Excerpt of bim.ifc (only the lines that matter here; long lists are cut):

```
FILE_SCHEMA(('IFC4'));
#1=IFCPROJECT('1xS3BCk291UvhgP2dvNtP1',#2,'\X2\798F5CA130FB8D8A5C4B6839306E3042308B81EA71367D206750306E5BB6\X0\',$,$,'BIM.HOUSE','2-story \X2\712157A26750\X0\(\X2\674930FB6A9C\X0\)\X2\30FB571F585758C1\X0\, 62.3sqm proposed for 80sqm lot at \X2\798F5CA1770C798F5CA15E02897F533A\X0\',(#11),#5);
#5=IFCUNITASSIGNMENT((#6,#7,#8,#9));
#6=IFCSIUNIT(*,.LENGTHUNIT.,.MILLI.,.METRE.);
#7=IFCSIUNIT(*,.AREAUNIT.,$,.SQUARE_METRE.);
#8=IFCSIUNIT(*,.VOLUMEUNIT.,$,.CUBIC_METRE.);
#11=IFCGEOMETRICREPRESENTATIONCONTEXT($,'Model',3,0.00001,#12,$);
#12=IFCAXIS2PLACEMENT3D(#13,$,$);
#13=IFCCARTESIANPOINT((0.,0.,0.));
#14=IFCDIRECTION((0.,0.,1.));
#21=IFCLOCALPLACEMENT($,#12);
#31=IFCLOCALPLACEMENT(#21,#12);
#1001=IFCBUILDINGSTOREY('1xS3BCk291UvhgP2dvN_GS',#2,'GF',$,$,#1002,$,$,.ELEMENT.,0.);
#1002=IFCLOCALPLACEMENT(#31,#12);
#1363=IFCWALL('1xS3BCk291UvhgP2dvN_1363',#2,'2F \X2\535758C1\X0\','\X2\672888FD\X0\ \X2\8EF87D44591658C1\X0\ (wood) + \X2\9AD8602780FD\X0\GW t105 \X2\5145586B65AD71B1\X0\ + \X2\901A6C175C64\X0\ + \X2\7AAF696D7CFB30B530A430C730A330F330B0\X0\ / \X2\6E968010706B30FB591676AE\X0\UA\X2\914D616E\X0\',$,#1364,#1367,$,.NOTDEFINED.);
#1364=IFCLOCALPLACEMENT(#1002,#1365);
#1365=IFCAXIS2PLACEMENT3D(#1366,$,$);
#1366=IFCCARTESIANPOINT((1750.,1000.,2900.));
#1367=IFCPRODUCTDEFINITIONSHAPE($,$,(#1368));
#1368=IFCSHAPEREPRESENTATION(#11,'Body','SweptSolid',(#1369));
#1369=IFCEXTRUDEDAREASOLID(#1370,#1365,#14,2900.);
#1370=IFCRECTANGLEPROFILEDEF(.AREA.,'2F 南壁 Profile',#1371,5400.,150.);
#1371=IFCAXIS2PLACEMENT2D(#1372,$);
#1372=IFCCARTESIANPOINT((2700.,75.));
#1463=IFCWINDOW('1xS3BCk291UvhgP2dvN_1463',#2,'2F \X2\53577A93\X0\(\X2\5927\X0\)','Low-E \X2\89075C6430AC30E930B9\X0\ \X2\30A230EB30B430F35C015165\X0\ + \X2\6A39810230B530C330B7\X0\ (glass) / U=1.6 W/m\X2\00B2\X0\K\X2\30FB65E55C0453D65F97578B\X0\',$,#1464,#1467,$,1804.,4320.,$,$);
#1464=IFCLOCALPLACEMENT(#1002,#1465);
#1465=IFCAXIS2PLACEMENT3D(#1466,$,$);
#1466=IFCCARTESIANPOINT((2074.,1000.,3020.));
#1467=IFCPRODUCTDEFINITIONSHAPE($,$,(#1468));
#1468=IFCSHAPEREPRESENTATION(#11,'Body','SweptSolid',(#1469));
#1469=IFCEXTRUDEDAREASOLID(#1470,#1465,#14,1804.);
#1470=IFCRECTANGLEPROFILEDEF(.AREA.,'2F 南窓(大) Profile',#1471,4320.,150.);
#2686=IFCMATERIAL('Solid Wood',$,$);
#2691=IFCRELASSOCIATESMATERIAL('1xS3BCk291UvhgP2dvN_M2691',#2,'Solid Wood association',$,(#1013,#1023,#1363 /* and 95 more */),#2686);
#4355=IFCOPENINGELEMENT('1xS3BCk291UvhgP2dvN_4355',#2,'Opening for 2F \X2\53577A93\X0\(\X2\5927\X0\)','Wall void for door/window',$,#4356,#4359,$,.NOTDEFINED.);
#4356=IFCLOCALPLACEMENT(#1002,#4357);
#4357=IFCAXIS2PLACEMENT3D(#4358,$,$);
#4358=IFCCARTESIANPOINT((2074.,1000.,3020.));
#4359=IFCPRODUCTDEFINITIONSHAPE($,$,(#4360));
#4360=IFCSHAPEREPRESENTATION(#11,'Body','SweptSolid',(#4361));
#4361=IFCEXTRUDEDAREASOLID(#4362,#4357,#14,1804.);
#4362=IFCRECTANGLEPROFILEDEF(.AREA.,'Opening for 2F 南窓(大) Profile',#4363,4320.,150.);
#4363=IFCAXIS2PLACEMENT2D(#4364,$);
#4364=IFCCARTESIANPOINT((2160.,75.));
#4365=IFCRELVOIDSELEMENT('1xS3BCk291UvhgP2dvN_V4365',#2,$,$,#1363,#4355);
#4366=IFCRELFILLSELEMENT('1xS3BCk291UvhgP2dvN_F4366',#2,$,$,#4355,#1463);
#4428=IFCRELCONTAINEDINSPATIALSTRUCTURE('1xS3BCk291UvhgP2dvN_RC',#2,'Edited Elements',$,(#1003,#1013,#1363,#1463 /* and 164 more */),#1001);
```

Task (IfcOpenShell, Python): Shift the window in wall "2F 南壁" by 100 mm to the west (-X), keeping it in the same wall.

```python
import ifcopenshell
import ifcopenshell.api.geometry
import ifcopenshell.util.placement

model = ifcopenshell.open("bim.ifc")

window = model.by_guid("1xS3BCk291UvhgP2dvN_1463")
opening = window.FillsVoids[0].RelatingOpeningElement
wall = opening.VoidsElements[0].RelatingBuildingElement

wall_matrix = ifcopenshell.util.placement.get_local_placement(wall.ObjectPlacement)
shift = wall_matrix[:3, 0] * -100.0
before = ifcopenshell.util.placement.get_local_placement(window.ObjectPlacement)[:3, 3].copy()

# The window is not placed relative to its opening, so move both.
for product in (opening, window):
    matrix = ifcopenshell.util.placement.get_local_placement(product.ObjectPlacement)
    matrix[:3, 3] += shift
    ifcopenshell.api.geometry.edit_object_placement(model, product=product, matrix=matrix, is_si=False)

after = ifcopenshell.util.placement.get_local_placement(window.ObjectPlacement)[:3, 3]
print("window moved by", (after - before).round(3) + 0.0)

model.write("bim_updated.ifc")
```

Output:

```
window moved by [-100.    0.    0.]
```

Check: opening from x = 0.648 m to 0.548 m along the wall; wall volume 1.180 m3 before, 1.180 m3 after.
